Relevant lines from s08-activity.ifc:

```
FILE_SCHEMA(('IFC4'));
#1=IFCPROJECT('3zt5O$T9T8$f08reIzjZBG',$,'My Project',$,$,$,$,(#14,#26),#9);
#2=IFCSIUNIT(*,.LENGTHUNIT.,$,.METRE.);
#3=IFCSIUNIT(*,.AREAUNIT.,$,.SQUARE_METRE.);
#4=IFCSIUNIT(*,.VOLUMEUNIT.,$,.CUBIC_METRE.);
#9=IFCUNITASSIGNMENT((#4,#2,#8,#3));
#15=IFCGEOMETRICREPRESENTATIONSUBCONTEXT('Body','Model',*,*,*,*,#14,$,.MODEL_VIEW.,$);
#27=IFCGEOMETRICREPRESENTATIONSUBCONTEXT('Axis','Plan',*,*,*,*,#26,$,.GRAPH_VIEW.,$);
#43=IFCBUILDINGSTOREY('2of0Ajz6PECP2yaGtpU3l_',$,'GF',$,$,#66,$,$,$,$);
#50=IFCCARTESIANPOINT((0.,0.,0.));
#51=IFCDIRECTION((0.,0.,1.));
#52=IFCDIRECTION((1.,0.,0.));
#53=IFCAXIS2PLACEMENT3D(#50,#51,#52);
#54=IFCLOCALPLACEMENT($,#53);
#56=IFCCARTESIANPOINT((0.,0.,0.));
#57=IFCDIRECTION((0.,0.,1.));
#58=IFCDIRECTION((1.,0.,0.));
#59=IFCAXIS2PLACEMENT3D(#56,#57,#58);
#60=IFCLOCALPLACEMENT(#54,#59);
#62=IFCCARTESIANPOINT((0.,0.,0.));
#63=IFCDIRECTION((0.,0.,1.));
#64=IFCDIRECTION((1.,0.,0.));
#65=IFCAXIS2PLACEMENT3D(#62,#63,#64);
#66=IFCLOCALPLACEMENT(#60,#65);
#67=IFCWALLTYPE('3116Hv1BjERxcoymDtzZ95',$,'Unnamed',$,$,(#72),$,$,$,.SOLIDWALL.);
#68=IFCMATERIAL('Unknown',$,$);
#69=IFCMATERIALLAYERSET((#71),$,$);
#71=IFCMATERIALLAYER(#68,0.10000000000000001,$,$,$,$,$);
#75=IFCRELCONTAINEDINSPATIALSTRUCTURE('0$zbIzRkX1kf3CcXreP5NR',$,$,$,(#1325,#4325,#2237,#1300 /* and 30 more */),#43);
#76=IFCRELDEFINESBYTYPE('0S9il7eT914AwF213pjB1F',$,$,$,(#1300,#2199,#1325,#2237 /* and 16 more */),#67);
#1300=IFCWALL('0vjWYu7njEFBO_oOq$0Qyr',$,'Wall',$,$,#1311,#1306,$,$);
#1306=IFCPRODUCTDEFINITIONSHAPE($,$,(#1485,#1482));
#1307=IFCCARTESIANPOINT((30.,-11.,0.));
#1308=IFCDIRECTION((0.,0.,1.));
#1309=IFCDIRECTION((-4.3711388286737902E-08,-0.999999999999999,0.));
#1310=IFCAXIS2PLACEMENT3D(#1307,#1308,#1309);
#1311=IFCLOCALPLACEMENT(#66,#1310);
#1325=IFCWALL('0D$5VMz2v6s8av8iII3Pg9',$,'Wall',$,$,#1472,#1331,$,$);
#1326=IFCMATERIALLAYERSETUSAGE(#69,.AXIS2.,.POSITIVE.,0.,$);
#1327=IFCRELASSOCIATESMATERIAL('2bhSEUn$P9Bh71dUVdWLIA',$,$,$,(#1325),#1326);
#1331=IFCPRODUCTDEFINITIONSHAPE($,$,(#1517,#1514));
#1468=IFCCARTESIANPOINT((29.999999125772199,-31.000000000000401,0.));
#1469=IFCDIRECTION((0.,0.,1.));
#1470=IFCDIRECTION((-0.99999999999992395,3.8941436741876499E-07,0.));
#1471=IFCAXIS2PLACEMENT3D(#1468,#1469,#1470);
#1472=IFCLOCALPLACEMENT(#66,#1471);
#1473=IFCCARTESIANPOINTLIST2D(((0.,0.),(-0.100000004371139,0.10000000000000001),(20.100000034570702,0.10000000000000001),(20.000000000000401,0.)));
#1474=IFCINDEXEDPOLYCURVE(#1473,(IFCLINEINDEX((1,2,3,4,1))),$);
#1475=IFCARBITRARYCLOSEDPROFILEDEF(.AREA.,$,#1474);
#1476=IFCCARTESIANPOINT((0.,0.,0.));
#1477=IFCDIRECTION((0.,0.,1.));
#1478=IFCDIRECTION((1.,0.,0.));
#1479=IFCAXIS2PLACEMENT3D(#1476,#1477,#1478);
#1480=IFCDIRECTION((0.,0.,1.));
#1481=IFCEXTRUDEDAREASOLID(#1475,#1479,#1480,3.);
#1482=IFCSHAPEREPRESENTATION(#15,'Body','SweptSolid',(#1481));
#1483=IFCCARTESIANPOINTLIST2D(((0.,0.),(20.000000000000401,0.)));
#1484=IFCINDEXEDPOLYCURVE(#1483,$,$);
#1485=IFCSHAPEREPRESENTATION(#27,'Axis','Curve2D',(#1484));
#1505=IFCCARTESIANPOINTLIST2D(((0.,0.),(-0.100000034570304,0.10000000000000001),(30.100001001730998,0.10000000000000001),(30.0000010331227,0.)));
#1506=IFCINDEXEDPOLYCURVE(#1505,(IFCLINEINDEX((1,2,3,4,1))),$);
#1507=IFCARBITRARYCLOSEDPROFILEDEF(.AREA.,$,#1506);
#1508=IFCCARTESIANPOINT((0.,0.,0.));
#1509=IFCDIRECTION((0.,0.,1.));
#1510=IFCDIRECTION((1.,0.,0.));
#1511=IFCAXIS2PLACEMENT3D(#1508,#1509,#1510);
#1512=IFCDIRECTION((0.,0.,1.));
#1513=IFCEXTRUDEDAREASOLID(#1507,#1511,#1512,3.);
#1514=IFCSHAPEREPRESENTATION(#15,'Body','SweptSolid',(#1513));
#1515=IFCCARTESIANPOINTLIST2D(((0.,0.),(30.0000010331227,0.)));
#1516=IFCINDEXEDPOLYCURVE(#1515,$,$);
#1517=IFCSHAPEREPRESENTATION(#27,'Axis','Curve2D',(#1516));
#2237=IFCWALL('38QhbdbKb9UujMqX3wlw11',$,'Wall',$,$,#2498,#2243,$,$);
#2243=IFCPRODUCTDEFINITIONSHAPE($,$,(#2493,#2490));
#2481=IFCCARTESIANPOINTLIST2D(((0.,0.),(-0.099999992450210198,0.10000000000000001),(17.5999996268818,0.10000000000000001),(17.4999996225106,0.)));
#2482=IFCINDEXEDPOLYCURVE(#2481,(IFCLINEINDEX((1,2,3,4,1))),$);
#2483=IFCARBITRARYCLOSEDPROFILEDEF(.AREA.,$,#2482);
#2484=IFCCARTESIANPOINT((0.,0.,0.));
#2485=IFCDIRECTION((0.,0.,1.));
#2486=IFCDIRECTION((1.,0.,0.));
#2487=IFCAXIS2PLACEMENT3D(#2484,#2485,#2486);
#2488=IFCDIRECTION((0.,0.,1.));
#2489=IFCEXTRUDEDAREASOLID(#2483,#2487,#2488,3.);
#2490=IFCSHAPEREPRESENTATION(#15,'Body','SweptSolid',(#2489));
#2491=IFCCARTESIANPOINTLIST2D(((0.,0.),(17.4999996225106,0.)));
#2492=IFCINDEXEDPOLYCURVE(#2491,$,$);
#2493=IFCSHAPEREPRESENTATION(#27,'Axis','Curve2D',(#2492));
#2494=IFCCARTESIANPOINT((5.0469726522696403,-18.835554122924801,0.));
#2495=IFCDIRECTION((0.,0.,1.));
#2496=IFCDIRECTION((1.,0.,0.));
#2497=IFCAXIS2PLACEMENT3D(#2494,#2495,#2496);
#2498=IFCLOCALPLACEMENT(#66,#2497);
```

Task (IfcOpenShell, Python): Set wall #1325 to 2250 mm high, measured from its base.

```python
import ifcopenshell
import ifcopenshell.geom
import ifcopenshell.util.representation
import ifcopenshell.util.shape
import ifcopenshell.util.unit

model = ifcopenshell.open("s08-activity.ifc")
unit_scale = ifcopenshell.util.unit.calculate_unit_scale(model)
settings = ifcopenshell.geom.settings()


def volume(element):
    """Net volume in cubic metres, openings subtracted."""
    shape = ifcopenshell.geom.create_shape(settings, element)
    return ifcopenshell.util.shape.get_volume(shape.geometry)


wall = model.by_id(1325)
before = volume(wall)

body = ifcopenshell.util.representation.get_representation(wall, "Model", "Body")
solid = body.Items[0]
old_height = solid.Depth
solid.Depth = 2.25 / unit_scale
after = volume(wall)

print(f"height {old_height:g} -> {solid.Depth:g}, volume {before:.3f} -> {after:.3f} m3")

model.write("s08-activity_v2.ifc")
```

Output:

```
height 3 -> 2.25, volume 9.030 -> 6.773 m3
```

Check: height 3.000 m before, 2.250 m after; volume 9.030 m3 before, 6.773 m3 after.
